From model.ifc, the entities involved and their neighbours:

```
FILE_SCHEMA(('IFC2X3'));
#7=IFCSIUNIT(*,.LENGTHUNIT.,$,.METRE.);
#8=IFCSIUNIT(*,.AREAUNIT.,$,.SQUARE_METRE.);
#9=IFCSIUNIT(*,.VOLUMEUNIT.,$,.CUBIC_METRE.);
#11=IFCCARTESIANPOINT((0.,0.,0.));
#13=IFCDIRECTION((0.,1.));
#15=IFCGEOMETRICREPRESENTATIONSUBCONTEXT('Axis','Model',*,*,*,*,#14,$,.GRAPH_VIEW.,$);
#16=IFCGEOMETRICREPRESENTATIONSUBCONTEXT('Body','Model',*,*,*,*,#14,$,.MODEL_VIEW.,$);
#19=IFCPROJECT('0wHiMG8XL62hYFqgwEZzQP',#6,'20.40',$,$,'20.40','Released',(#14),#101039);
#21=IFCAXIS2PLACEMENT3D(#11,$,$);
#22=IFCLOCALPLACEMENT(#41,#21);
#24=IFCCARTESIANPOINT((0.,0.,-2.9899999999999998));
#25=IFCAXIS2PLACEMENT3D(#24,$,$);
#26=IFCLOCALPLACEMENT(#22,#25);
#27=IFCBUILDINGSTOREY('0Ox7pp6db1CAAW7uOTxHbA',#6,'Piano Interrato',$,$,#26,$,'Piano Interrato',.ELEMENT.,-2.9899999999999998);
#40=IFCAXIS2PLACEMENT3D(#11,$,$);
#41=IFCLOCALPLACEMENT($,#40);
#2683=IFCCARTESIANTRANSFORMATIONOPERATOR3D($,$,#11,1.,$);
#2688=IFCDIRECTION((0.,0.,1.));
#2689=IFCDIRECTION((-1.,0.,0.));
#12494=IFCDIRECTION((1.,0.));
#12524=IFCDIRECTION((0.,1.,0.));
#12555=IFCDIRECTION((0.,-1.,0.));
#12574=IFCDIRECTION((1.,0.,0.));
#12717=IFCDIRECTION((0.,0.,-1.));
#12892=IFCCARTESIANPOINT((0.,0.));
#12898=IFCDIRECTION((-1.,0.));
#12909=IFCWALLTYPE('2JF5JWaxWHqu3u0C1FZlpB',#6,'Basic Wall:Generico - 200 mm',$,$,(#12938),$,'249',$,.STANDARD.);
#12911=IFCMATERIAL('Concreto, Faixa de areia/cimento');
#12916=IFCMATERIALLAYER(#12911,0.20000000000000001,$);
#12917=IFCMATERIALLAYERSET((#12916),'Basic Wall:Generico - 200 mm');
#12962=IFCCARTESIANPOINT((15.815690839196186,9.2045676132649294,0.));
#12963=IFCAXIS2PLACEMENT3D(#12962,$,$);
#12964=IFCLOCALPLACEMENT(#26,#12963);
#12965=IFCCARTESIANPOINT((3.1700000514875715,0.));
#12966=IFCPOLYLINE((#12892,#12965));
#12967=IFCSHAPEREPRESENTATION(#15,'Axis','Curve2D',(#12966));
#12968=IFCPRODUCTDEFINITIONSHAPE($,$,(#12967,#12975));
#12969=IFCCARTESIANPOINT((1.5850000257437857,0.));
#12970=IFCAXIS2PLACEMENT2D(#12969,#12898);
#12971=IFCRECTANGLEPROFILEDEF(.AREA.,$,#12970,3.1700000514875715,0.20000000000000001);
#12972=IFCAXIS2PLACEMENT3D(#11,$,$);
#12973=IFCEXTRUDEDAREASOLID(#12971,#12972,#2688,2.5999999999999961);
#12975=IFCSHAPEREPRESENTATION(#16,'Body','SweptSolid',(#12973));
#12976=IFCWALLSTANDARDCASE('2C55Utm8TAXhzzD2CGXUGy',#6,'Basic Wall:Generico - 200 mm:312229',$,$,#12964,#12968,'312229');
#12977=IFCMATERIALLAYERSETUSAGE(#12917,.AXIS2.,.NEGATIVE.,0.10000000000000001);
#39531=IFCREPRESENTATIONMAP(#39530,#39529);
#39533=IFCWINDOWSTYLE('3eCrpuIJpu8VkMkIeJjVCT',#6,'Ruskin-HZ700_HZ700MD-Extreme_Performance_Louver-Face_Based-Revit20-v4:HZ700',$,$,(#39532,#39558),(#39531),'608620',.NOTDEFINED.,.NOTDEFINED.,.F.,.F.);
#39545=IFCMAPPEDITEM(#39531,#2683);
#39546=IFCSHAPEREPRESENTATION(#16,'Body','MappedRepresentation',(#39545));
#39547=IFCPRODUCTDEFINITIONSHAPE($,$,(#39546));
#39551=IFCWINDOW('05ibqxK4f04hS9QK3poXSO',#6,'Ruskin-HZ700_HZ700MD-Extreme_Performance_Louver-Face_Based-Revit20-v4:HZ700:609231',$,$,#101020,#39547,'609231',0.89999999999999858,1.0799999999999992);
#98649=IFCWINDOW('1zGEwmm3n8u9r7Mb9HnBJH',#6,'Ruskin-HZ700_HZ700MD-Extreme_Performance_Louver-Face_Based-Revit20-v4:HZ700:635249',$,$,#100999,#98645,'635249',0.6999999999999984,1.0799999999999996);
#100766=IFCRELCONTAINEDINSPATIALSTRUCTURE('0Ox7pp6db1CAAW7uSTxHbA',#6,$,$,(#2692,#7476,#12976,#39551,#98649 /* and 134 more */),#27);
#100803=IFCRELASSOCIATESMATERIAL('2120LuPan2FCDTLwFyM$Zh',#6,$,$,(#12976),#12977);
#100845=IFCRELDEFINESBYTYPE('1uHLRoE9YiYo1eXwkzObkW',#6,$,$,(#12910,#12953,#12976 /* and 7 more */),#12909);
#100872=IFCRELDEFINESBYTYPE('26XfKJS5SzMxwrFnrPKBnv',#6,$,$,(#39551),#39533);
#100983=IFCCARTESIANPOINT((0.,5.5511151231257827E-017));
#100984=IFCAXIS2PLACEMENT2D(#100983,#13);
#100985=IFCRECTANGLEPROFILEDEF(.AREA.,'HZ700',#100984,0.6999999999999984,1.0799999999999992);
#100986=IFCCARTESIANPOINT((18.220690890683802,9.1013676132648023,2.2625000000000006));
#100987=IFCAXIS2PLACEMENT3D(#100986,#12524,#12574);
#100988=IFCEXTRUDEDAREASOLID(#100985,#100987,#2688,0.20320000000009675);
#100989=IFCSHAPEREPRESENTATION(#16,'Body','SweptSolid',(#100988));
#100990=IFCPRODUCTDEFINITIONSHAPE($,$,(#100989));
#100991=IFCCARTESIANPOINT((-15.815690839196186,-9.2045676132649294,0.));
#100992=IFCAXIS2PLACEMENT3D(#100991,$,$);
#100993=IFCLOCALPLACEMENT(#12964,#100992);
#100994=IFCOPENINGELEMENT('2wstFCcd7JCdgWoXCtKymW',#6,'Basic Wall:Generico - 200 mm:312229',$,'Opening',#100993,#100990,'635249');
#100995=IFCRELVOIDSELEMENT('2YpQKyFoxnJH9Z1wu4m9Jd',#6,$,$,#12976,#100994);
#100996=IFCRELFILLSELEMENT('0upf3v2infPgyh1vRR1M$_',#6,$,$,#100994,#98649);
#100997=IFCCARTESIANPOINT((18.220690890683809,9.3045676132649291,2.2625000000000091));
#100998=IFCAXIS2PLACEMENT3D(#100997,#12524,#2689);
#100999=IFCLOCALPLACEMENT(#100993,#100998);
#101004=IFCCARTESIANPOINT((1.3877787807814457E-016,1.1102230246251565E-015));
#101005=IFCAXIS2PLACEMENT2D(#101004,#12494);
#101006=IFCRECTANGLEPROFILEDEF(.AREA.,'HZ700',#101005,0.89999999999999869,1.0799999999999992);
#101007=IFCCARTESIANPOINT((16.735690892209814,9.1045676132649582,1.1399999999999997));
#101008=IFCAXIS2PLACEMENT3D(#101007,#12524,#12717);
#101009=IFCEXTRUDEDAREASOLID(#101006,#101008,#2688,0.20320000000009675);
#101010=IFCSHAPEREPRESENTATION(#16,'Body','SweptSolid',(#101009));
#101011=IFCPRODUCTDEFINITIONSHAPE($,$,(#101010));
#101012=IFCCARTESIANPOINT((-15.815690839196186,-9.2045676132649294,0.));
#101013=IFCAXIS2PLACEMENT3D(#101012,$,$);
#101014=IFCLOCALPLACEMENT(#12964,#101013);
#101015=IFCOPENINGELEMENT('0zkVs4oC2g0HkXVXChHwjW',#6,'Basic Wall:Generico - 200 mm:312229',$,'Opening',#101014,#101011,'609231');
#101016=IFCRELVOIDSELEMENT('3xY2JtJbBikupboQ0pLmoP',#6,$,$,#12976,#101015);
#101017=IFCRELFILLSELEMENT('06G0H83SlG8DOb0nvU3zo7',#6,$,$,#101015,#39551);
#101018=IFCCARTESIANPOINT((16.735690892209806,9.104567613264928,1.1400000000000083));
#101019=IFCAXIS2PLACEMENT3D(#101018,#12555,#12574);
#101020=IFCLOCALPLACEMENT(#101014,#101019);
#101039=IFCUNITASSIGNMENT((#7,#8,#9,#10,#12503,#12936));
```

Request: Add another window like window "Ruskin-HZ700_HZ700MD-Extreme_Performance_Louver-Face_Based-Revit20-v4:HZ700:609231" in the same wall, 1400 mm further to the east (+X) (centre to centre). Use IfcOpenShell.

```python
import ifcopenshell
import ifcopenshell.api.feature
import ifcopenshell.api.geometry
import ifcopenshell.api.root
import ifcopenshell.geom
import ifcopenshell.util.element
import ifcopenshell.util.placement
import ifcopenshell.util.shape
import ifcopenshell.util.unit

model = ifcopenshell.open("model.ifc")
unit_scale = ifcopenshell.util.unit.calculate_unit_scale(model)
settings = ifcopenshell.geom.settings()


def volume(element):
    """Net volume in cubic metres, openings subtracted."""
    shape = ifcopenshell.geom.create_shape(settings, element)
    return ifcopenshell.util.shape.get_volume(shape.geometry)


def reuse_history(source, copy):
    """copy_class also copies each property set's owner history, people and application; keep the originals."""
    for rel in copy.IsDefinedBy:
        if rel.is_a("IfcRelDefinesByProperties") and (history := rel.RelatingPropertyDefinition.OwnerHistory):
            rel.RelatingPropertyDefinition.OwnerHistory = source.OwnerHistory
            ifcopenshell.util.element.remove_deep2(model, history)


window = model.by_guid("05ibqxK4f04hS9QK3poXSO")
opening = window.FillsVoids[0].RelatingOpeningElement
wall = opening.VoidsElements[0].RelatingBuildingElement
before = volume(wall)
shift = ifcopenshell.util.placement.get_local_placement(wall.ObjectPlacement)[:3, 0] * 1.4 / unit_scale

# copy_class copies the void relationship, type, container and properties, but no geometry.
new_opening = ifcopenshell.api.root.copy_class(model, product=opening)
new_opening.Representation = ifcopenshell.util.element.copy_deep(
    model, opening.Representation, exclude=["IfcGeometricRepresentationContext", "IfcRepresentationMap"]
)
new_opening.Name = "Basic Wall:Generico - 200 mm"
new_opening.Tag = None
new_window = ifcopenshell.api.root.copy_class(model, product=window)
new_window.Representation = ifcopenshell.util.element.copy_deep(
    model, window.Representation, exclude=["IfcGeometricRepresentationContext", "IfcRepresentationMap"]
)
new_window.Name = "Ruskin-HZ700_HZ700MD-Extreme_Performance_Louver-Face_Based-Revit20-v4:HZ700"
new_window.Tag = None
reuse_history(window, new_window)
fills = ifcopenshell.api.feature.add_filling(model, opening=new_opening, element=new_window)
fills.OwnerHistory = new_window.OwnerHistory  # required in IFC2X3

for old, new in ((opening, new_opening), (window, new_window)):
    matrix = ifcopenshell.util.placement.get_local_placement(old.ObjectPlacement)
    matrix[:3, 3] += shift
    ifcopenshell.api.geometry.edit_object_placement(model, product=new, matrix=matrix, is_si=False)

after = volume(wall)

print(f"wall volume {before:.3f} -> {after:.3f} m3")

model.write("model_updated.ifc")
```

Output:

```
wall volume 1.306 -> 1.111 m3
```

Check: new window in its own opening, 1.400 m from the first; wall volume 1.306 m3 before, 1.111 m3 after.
